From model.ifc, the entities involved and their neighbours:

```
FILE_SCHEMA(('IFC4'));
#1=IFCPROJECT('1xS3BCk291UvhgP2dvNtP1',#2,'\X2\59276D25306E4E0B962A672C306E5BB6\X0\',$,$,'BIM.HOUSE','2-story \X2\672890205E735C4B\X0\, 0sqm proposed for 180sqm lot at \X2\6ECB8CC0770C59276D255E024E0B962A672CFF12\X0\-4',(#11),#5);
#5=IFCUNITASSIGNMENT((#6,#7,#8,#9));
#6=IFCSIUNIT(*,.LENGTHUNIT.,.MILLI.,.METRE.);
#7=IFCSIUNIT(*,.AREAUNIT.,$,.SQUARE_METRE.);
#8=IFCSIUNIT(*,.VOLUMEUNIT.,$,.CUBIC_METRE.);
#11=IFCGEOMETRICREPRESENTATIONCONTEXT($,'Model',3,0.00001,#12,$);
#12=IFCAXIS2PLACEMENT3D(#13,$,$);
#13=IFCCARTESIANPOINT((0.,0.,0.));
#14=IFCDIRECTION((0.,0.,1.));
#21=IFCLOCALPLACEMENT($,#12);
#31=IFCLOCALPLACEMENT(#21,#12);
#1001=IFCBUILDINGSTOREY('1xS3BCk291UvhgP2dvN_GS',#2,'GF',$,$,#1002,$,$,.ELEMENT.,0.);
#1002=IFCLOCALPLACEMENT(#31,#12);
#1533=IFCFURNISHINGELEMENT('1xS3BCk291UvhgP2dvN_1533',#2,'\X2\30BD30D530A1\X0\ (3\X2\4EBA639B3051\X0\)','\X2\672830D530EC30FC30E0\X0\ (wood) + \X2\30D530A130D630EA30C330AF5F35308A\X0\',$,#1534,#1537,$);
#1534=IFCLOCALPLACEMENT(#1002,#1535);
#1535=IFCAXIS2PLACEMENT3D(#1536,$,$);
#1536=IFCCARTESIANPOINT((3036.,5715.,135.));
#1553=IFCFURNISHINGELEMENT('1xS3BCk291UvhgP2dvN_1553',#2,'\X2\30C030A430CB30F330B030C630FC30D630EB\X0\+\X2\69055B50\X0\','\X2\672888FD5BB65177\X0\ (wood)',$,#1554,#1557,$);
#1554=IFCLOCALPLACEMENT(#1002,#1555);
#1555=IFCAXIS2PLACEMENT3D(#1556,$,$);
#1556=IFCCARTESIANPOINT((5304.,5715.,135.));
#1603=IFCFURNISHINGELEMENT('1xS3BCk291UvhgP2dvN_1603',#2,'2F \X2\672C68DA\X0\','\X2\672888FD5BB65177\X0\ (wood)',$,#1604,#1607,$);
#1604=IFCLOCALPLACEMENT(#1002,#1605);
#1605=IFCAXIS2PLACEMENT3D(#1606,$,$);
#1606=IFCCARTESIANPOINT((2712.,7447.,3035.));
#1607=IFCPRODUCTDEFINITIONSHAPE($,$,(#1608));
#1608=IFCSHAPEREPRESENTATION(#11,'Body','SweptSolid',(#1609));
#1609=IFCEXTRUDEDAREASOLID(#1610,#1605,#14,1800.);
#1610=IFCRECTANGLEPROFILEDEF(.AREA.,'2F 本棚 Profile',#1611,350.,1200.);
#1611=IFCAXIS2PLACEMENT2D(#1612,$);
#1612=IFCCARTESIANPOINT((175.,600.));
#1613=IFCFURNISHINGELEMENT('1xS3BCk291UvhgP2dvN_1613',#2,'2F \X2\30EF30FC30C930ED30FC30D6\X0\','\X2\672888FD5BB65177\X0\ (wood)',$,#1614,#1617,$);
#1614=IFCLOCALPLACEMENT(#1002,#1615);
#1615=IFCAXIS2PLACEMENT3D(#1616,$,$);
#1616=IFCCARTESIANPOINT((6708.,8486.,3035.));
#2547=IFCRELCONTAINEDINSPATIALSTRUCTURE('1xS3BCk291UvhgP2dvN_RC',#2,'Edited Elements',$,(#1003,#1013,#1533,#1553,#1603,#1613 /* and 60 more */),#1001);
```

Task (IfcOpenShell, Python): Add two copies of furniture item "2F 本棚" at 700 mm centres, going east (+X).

```python
import numpy as np
import ifcopenshell
import ifcopenshell.api.geometry
import ifcopenshell.api.root
import ifcopenshell.util.element
import ifcopenshell.util.placement

model = ifcopenshell.open("model.ifc")


def reuse_history(source, copy):
    """copy_class also copies each property set's owner history, people and application; keep the originals."""
    for rel in copy.IsDefinedBy:
        if rel.is_a("IfcRelDefinesByProperties") and (history := rel.RelatingPropertyDefinition.OwnerHistory):
            rel.RelatingPropertyDefinition.OwnerHistory = source.OwnerHistory
            ifcopenshell.util.element.remove_deep2(model, history)


source = model.by_guid("1xS3BCk291UvhgP2dvN_1603")
base = ifcopenshell.util.placement.get_local_placement(source.ObjectPlacement)
step = np.array([1.0, 0.0, 0.0]) * 700.0

for i in range(1, 3):
    copy = ifcopenshell.api.root.copy_class(model, product=source)
    copy.Representation = ifcopenshell.util.element.copy_deep(
        model, source.Representation, exclude=["IfcGeometricRepresentationContext", "IfcRepresentationMap"]
    )
    reuse_history(source, copy)
    matrix = base.copy()
    matrix[:3, 3] += i * step
    print("added at", matrix[:3, 3].round(3) + 0.0)
    ifcopenshell.api.geometry.edit_object_placement(model, product=copy, matrix=matrix, is_si=False)

model.write("model_edited.ifc")
```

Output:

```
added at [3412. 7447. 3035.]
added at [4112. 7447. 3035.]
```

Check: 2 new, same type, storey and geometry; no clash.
